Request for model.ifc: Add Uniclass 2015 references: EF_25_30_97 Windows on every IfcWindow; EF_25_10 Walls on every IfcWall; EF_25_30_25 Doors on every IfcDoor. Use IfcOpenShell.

First a look at what the model holds.

```python
import ifcopenshell

model = ifcopenshell.open("model.ifc")
print(model.schema)
print("classifications:", [c.Name for c in model.by_type("IfcClassification")])
for ifc_class in ("IfcDoor", "IfcRoof", "IfcStair", "IfcWall", "IfcWindow"):
    print(ifc_class, len(model.by_type(ifc_class)))
```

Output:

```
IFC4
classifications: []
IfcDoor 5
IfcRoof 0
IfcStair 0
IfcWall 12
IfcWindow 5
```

```python
import ifcopenshell
import ifcopenshell.api.classification

model = ifcopenshell.open("model.ifc")

system = ifcopenshell.api.classification.add_classification(model, classification="Uniclass 2015")

codes = {
    "IfcWindow": ("EF_25_30_97", "Windows"),
    "IfcWall": ("EF_25_10", "Walls"),
    "IfcDoor": ("EF_25_30_25", "Doors"),
}
for ifc_class, (code, name) in codes.items():
    products = model.by_type(ifc_class)
    ifcopenshell.api.classification.add_reference(
        model, products=products, classification=system, identification=code, name=name
    )
    print(code, len(products))

model.write("model_rev.ifc")
```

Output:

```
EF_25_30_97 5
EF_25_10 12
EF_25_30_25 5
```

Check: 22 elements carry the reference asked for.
